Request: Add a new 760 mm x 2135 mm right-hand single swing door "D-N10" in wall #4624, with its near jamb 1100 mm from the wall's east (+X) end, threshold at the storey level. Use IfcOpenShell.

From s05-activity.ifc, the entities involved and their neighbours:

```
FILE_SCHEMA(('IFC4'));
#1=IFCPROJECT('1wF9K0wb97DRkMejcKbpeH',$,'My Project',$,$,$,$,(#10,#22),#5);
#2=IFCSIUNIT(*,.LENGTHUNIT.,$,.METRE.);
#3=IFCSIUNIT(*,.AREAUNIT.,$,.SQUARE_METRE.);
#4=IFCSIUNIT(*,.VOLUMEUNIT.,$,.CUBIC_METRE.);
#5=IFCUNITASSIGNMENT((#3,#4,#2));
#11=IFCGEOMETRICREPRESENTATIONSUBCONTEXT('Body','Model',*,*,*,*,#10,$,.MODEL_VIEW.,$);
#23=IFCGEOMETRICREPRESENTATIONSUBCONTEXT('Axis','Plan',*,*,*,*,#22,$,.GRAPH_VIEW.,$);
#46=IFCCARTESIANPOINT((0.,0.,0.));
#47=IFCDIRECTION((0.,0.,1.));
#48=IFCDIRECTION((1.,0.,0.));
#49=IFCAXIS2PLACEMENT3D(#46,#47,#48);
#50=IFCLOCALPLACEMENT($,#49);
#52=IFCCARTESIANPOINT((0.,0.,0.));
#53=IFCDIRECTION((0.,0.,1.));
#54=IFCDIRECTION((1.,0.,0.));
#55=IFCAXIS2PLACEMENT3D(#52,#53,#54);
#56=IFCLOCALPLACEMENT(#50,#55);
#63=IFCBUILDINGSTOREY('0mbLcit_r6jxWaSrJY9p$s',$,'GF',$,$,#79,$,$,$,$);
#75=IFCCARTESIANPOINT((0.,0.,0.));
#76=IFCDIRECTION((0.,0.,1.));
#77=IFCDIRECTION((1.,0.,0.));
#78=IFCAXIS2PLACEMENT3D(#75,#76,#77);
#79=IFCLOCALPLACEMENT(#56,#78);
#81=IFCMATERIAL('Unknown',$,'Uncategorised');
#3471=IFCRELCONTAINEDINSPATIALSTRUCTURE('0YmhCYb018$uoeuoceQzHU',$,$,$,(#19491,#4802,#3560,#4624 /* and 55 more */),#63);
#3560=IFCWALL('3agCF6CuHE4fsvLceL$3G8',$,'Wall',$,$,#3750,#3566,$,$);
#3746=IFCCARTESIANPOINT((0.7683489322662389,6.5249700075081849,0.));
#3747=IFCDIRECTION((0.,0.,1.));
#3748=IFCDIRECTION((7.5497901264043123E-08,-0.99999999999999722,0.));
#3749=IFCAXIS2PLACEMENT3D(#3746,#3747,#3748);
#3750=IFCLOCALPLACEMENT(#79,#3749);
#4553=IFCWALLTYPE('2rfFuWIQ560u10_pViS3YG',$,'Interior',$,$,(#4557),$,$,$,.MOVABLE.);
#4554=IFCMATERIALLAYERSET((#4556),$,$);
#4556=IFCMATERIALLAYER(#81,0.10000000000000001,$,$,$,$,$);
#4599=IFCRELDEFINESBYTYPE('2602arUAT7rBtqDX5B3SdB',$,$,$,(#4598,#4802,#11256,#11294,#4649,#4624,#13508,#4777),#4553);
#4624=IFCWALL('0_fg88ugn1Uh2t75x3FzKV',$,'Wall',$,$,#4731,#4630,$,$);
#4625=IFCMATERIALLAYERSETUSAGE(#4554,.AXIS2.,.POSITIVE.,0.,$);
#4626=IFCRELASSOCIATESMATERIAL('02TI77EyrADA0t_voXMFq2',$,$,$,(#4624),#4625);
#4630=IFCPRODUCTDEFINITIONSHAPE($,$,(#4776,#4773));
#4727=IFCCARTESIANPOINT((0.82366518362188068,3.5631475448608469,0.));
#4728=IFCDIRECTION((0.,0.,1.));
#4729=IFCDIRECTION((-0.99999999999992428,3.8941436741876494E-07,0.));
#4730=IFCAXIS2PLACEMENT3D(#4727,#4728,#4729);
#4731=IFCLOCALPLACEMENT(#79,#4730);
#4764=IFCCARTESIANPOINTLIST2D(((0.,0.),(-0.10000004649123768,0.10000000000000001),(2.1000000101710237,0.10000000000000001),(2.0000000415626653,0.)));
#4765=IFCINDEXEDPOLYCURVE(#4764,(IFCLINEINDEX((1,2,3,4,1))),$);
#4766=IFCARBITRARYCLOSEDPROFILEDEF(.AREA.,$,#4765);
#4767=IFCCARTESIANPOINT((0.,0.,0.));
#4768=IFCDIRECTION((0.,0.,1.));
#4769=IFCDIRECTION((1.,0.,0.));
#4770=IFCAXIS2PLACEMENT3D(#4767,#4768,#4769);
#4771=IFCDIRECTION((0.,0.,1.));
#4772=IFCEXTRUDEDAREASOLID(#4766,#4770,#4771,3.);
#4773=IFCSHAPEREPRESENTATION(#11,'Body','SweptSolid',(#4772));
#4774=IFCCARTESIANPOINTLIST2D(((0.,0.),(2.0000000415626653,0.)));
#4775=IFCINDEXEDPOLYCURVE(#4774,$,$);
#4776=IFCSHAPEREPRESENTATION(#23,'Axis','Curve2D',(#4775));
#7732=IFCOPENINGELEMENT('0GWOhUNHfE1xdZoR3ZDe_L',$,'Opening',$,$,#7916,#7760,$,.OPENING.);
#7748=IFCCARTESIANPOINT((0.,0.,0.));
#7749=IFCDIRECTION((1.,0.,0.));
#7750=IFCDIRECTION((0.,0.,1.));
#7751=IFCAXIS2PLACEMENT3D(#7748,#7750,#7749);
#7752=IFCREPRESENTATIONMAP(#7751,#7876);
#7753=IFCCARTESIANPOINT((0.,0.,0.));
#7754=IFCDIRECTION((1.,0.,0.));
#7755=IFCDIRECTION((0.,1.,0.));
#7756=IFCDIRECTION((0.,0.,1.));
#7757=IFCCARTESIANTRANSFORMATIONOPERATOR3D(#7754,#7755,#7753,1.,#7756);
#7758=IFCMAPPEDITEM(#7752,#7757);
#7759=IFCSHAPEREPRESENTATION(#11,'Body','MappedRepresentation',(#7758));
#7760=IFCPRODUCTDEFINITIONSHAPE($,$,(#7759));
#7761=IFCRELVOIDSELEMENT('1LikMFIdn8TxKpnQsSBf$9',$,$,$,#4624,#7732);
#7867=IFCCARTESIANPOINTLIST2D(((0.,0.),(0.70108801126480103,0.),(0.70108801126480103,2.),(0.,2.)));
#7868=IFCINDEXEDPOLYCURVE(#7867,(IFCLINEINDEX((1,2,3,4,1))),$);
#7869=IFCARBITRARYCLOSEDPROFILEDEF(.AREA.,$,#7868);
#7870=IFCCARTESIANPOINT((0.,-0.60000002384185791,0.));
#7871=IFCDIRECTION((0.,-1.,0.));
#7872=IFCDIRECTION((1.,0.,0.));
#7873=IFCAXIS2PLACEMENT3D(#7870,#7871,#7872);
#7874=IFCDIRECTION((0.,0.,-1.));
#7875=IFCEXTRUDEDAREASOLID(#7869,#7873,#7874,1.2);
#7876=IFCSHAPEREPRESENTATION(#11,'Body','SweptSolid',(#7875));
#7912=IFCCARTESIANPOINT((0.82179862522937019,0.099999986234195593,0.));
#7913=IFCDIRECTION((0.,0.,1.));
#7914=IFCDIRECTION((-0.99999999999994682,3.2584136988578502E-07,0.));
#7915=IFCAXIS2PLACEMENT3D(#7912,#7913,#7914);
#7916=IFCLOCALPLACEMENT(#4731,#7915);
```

```python
import numpy as np
import ifcopenshell
import ifcopenshell.api.feature
import ifcopenshell.api.geometry
import ifcopenshell.api.root
import ifcopenshell.api.spatial
import ifcopenshell.geom
import ifcopenshell.util.element
import ifcopenshell.util.placement
import ifcopenshell.util.representation
import ifcopenshell.util.shape
import ifcopenshell.util.unit

model = ifcopenshell.open("s05-activity.ifc")
unit_scale = ifcopenshell.util.unit.calculate_unit_scale(model)
settings = ifcopenshell.geom.settings()


def volume(element):
    """Net volume in cubic metres, openings subtracted."""
    shape = ifcopenshell.geom.create_shape(settings, element)
    return ifcopenshell.util.shape.get_volume(shape.geometry)


wall = model.by_guid("0_fg88ugn1Uh2t75x3FzKV")
storey = ifcopenshell.util.element.get_container(wall, ifc_class="IfcBuildingStorey")
context = ifcopenshell.util.representation.get_context(model, "Model", "Body", "MODEL_VIEW")
before = volume(wall)

width, height, from_end, sill = 0.76, 2.135, 1.1, 0.0  # metres

# The wall runs along its own X axis, and the end named is its -X end.
wall_shape = ifcopenshell.geom.create_shape(settings, wall)
x, y, z = ifcopenshell.util.shape.get_vertices(wall_shape.geometry).T
start = x.min() + from_end
face, thickness = float(y.min()), float(y.max() - y.min())
wall_matrix = ifcopenshell.util.placement.get_local_placement(wall.ObjectPlacement)
level = ifcopenshell.util.placement.get_local_placement(storey.ObjectPlacement)[2, 3]


def in_wall(x, y):
    """Placement at x, y metres in the wall's axes, at sill height."""
    matrix = wall_matrix.copy()
    matrix[:, 3] = wall_matrix @ np.array([x / unit_scale, y / unit_scale, 0.0, 1.0])
    matrix[2, 3] = level + sill / unit_scale
    return matrix


# Opening: a box that overshoots both wall faces by 50 mm.
opening = ifcopenshell.api.root.create_entity(model, ifc_class="IfcOpeningElement", predefined_type="OPENING")
box = ifcopenshell.api.geometry.add_wall_representation(
    model, context=context, length=width, height=height, thickness=thickness + 0.1
)
ifcopenshell.api.geometry.assign_representation(model, product=opening, representation=box)
ifcopenshell.api.geometry.edit_object_placement(model, product=opening, matrix=in_wall(start, face - 0.05), is_si=False)
ifcopenshell.api.feature.add_feature(model, feature=opening, element=wall)

door = ifcopenshell.api.root.create_entity(model, ifc_class="IfcDoor", name="D-N10", predefined_type="DOOR")
door.OverallWidth, door.OverallHeight = width / unit_scale, height / unit_scale
door.OperationType = "SINGLE_SWING_RIGHT"
body = ifcopenshell.api.geometry.add_door_representation(
    model,
    context=context,
    overall_width=door.OverallWidth,
    overall_height=door.OverallHeight,
    operation_type="SINGLE_SWING_RIGHT",
    lining_properties={"LiningDepth": thickness / unit_scale, "ThresholdDepth": thickness / unit_scale},
)
ifcopenshell.api.geometry.assign_representation(model, product=door, representation=body)
ifcopenshell.api.spatial.assign_container(model, products=[door], relating_structure=storey)
ifcopenshell.api.feature.add_filling(model, opening=opening, element=door)

# The lining spans the wall, so the door starts at the wall face.
ifcopenshell.api.geometry.edit_object_placement(model, product=door, matrix=in_wall(start, face), is_si=False)

after = volume(wall)

print(f"wall volume {before:.3f} -> {after:.3f} m3")

model.write("s05-activity_edited.ifc")
```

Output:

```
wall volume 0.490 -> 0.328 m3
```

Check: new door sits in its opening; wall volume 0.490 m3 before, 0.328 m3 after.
